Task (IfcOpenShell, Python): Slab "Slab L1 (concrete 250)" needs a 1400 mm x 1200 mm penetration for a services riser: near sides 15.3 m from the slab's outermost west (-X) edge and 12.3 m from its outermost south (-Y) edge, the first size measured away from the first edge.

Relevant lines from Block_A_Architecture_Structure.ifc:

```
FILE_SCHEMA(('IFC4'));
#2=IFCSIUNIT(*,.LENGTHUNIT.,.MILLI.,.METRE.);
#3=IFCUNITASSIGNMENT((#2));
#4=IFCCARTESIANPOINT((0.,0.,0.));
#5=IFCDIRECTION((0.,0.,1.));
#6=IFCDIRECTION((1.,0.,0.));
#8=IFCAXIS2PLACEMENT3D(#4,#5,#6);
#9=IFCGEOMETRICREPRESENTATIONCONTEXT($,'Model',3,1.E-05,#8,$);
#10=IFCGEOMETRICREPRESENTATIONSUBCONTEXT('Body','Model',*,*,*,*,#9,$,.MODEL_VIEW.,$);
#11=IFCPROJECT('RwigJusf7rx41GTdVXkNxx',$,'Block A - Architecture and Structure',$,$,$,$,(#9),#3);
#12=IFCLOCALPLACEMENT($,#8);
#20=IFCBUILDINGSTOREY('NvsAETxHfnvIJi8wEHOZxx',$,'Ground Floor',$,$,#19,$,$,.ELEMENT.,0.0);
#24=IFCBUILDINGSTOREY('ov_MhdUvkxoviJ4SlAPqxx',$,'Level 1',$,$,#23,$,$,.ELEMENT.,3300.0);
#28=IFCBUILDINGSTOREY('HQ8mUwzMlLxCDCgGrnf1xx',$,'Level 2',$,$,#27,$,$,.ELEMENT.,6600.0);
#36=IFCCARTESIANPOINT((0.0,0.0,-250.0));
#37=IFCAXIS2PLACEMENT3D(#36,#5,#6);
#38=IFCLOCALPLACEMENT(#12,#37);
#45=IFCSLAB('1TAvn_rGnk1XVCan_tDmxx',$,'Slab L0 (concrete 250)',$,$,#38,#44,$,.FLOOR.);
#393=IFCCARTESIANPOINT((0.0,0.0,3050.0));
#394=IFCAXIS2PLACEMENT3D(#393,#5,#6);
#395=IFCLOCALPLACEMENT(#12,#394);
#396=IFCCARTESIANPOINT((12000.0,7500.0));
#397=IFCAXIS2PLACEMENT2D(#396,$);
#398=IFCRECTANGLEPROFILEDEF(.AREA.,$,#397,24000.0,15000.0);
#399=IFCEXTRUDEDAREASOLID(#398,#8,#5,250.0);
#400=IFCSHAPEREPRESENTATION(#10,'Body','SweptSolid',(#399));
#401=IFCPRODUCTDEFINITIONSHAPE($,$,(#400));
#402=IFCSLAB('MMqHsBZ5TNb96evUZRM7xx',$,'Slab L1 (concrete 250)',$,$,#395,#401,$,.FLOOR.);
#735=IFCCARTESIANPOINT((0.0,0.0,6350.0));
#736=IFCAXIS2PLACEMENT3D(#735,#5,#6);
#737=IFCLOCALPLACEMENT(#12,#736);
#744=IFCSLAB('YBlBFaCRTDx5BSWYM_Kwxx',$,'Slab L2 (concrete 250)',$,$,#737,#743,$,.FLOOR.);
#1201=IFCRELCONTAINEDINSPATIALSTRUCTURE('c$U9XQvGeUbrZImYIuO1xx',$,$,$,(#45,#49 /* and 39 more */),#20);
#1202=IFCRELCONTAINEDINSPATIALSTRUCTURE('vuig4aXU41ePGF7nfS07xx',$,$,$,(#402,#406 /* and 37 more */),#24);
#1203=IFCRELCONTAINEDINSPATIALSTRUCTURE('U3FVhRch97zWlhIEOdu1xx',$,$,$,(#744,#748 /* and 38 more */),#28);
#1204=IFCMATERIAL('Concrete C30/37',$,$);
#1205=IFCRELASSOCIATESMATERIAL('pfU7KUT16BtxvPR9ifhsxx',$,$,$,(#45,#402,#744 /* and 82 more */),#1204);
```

```python
import numpy as np
import ifcopenshell
import ifcopenshell.api.feature
import ifcopenshell.api.geometry
import ifcopenshell.api.root
import ifcopenshell.geom
import ifcopenshell.util.placement
import ifcopenshell.util.representation
import ifcopenshell.util.shape
import ifcopenshell.util.unit

model = ifcopenshell.open("Block_A_Architecture_Structure.ifc")
unit_scale = ifcopenshell.util.unit.calculate_unit_scale(model)
settings = ifcopenshell.geom.settings()


def volume(element):
    """Net volume in cubic metres, openings subtracted."""
    shape = ifcopenshell.geom.create_shape(settings, element)
    return ifcopenshell.util.shape.get_volume(shape.geometry)


slab = model.by_guid("MMqHsBZ5TNb96evUZRM7xx")
before = volume(slab)

# Extent in the slab's own axes, in metres. The edges named are its -X and -Y sides.
slab_shape = ifcopenshell.geom.create_shape(settings, slab)
vertices = ifcopenshell.util.shape.get_vertices(slab_shape.geometry)
x_min, y_min, bottom = vertices.min(axis=0)
top = vertices[:, 2].max()

opening = ifcopenshell.api.root.create_entity(model, ifc_class="IfcOpeningElement", name="Services riser opening", predefined_type="OPENING")
context = ifcopenshell.util.representation.get_context(model, "Model", "Body", "MODEL_VIEW")
width, depth = 1.4, 1.2
outline = [(0.0, 0.0), (width, 0.0), (width, depth), (0.0, depth), (0.0, 0.0)]
# Overshoot both faces by 50 mm so the cut is clean.
shape = ifcopenshell.api.geometry.add_slab_representation(
    model, context=context, depth=top - bottom + 0.1, polyline=outline
)
ifcopenshell.api.geometry.assign_representation(model, product=opening, representation=shape)

matrix = ifcopenshell.util.placement.get_local_placement(slab.ObjectPlacement)
matrix[:, 3] = matrix @ np.append(np.array([x_min + 15.3, y_min + 12.3, bottom - 0.05]) / unit_scale, 1.0)
ifcopenshell.api.geometry.edit_object_placement(model, product=opening, matrix=matrix, is_si=False)
ifcopenshell.api.feature.add_feature(model, feature=opening, element=slab)

after = volume(slab)

print(f"slab volume {before:.3f} -> {after:.3f} m3")

model.write("Block_A_Architecture_Structure-out.ifc")
```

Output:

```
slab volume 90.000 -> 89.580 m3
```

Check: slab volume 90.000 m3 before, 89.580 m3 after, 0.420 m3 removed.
